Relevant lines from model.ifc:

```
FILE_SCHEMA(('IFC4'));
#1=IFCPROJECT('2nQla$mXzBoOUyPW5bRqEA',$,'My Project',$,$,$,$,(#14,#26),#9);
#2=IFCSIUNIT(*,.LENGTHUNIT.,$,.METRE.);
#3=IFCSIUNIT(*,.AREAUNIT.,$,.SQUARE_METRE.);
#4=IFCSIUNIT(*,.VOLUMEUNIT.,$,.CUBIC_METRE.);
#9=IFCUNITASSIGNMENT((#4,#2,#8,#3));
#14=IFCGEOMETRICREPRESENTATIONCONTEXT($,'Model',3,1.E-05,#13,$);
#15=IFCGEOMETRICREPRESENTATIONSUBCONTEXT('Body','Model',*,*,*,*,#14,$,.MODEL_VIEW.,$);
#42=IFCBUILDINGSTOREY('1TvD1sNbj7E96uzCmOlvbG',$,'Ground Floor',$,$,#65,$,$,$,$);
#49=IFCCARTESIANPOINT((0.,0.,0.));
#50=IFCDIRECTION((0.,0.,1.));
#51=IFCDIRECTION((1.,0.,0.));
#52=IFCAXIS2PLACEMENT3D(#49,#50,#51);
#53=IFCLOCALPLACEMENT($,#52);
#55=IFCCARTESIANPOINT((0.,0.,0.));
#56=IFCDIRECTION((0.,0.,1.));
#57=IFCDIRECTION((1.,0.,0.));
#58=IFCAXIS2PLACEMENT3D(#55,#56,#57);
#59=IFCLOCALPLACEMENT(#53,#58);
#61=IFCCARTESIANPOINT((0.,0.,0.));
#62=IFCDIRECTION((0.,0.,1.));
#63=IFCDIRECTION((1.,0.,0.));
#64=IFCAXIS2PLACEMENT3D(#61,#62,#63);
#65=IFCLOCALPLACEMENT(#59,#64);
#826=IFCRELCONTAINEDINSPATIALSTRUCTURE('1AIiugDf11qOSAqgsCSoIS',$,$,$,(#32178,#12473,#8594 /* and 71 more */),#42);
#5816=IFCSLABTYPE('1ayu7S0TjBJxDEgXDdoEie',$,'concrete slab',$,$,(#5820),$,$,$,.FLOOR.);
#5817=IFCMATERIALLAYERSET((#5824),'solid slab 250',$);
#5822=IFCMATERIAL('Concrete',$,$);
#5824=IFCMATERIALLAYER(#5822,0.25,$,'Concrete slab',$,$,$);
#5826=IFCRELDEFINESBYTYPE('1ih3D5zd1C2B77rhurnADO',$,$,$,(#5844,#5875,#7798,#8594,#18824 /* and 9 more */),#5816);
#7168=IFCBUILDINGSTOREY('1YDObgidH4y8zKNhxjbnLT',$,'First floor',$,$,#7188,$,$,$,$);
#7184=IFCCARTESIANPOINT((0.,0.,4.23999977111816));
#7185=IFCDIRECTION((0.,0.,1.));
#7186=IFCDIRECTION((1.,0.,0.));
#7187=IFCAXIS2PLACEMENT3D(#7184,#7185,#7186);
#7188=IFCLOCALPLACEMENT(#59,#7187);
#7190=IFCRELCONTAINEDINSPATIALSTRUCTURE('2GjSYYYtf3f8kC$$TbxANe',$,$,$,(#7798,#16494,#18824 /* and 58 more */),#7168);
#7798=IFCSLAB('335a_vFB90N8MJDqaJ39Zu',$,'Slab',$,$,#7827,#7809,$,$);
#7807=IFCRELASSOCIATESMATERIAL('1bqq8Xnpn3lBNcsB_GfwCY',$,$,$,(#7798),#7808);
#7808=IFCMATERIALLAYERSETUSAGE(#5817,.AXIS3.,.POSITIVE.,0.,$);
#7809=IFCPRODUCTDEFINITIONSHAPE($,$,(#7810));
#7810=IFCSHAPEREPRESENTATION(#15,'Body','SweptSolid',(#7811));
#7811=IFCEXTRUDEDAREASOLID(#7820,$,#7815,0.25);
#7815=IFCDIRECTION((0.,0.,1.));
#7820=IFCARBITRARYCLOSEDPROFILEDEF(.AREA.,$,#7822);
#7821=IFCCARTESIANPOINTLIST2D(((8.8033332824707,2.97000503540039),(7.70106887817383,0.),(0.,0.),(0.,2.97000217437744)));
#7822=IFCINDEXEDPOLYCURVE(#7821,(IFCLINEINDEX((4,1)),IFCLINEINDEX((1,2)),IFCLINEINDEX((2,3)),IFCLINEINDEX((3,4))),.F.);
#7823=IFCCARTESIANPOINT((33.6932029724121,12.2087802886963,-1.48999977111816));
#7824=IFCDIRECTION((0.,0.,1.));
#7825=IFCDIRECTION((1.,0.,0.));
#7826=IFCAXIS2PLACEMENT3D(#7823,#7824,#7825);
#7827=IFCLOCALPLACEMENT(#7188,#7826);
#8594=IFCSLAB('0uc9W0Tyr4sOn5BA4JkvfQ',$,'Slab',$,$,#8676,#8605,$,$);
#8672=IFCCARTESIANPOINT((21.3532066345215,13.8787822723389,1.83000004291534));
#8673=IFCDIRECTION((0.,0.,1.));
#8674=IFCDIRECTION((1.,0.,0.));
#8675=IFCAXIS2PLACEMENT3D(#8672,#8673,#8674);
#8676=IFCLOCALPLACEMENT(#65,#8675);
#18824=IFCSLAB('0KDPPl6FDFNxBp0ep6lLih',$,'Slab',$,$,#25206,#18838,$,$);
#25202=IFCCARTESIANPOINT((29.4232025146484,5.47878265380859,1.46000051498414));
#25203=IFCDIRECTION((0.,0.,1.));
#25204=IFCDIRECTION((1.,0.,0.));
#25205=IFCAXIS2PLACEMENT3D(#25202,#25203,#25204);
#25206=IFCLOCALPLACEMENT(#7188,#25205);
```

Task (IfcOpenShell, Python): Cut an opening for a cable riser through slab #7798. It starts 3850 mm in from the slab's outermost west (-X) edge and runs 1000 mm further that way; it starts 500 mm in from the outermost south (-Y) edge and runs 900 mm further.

```python
import numpy as np
import ifcopenshell
import ifcopenshell.api.feature
import ifcopenshell.api.geometry
import ifcopenshell.api.root
import ifcopenshell.geom
import ifcopenshell.util.placement
import ifcopenshell.util.representation
import ifcopenshell.util.shape
import ifcopenshell.util.unit

model = ifcopenshell.open("model.ifc")
unit_scale = ifcopenshell.util.unit.calculate_unit_scale(model)
settings = ifcopenshell.geom.settings()


def volume(element):
    """Net volume in cubic metres, openings subtracted."""
    shape = ifcopenshell.geom.create_shape(settings, element)
    return ifcopenshell.util.shape.get_volume(shape.geometry)


slab = model.by_guid("335a_vFB90N8MJDqaJ39Zu")
before = volume(slab)

# Extent in the slab's own axes, in metres. The edges named are its -X and -Y sides.
slab_shape = ifcopenshell.geom.create_shape(settings, slab)
vertices = ifcopenshell.util.shape.get_vertices(slab_shape.geometry)
x_min, y_min, bottom = vertices.min(axis=0)
top = vertices[:, 2].max()

opening = ifcopenshell.api.root.create_entity(model, ifc_class="IfcOpeningElement", name="Cable riser opening", predefined_type="OPENING")
context = ifcopenshell.util.representation.get_context(model, "Model", "Body", "MODEL_VIEW")
width, depth = 1, 0.9
outline = [(0.0, 0.0), (width, 0.0), (width, depth), (0.0, depth), (0.0, 0.0)]
# Overshoot both faces by 50 mm so the cut is clean.
shape = ifcopenshell.api.geometry.add_slab_representation(
    model, context=context, depth=top - bottom + 0.1, polyline=outline
)
ifcopenshell.api.geometry.assign_representation(model, product=opening, representation=shape)

matrix = ifcopenshell.util.placement.get_local_placement(slab.ObjectPlacement)
matrix[:, 3] = matrix @ np.append(np.array([x_min + 3.85, y_min + 0.5, bottom - 0.05]) / unit_scale, 1.0)
ifcopenshell.api.geometry.edit_object_placement(model, product=opening, matrix=matrix, is_si=False)
ifcopenshell.api.feature.add_feature(model, feature=opening, element=slab)

after = volume(slab)

print(f"slab volume {before:.3f} -> {after:.3f} m3")

model.write("model-out.ifc")
```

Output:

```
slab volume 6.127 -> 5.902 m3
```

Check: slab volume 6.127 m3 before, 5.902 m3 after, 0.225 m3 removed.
